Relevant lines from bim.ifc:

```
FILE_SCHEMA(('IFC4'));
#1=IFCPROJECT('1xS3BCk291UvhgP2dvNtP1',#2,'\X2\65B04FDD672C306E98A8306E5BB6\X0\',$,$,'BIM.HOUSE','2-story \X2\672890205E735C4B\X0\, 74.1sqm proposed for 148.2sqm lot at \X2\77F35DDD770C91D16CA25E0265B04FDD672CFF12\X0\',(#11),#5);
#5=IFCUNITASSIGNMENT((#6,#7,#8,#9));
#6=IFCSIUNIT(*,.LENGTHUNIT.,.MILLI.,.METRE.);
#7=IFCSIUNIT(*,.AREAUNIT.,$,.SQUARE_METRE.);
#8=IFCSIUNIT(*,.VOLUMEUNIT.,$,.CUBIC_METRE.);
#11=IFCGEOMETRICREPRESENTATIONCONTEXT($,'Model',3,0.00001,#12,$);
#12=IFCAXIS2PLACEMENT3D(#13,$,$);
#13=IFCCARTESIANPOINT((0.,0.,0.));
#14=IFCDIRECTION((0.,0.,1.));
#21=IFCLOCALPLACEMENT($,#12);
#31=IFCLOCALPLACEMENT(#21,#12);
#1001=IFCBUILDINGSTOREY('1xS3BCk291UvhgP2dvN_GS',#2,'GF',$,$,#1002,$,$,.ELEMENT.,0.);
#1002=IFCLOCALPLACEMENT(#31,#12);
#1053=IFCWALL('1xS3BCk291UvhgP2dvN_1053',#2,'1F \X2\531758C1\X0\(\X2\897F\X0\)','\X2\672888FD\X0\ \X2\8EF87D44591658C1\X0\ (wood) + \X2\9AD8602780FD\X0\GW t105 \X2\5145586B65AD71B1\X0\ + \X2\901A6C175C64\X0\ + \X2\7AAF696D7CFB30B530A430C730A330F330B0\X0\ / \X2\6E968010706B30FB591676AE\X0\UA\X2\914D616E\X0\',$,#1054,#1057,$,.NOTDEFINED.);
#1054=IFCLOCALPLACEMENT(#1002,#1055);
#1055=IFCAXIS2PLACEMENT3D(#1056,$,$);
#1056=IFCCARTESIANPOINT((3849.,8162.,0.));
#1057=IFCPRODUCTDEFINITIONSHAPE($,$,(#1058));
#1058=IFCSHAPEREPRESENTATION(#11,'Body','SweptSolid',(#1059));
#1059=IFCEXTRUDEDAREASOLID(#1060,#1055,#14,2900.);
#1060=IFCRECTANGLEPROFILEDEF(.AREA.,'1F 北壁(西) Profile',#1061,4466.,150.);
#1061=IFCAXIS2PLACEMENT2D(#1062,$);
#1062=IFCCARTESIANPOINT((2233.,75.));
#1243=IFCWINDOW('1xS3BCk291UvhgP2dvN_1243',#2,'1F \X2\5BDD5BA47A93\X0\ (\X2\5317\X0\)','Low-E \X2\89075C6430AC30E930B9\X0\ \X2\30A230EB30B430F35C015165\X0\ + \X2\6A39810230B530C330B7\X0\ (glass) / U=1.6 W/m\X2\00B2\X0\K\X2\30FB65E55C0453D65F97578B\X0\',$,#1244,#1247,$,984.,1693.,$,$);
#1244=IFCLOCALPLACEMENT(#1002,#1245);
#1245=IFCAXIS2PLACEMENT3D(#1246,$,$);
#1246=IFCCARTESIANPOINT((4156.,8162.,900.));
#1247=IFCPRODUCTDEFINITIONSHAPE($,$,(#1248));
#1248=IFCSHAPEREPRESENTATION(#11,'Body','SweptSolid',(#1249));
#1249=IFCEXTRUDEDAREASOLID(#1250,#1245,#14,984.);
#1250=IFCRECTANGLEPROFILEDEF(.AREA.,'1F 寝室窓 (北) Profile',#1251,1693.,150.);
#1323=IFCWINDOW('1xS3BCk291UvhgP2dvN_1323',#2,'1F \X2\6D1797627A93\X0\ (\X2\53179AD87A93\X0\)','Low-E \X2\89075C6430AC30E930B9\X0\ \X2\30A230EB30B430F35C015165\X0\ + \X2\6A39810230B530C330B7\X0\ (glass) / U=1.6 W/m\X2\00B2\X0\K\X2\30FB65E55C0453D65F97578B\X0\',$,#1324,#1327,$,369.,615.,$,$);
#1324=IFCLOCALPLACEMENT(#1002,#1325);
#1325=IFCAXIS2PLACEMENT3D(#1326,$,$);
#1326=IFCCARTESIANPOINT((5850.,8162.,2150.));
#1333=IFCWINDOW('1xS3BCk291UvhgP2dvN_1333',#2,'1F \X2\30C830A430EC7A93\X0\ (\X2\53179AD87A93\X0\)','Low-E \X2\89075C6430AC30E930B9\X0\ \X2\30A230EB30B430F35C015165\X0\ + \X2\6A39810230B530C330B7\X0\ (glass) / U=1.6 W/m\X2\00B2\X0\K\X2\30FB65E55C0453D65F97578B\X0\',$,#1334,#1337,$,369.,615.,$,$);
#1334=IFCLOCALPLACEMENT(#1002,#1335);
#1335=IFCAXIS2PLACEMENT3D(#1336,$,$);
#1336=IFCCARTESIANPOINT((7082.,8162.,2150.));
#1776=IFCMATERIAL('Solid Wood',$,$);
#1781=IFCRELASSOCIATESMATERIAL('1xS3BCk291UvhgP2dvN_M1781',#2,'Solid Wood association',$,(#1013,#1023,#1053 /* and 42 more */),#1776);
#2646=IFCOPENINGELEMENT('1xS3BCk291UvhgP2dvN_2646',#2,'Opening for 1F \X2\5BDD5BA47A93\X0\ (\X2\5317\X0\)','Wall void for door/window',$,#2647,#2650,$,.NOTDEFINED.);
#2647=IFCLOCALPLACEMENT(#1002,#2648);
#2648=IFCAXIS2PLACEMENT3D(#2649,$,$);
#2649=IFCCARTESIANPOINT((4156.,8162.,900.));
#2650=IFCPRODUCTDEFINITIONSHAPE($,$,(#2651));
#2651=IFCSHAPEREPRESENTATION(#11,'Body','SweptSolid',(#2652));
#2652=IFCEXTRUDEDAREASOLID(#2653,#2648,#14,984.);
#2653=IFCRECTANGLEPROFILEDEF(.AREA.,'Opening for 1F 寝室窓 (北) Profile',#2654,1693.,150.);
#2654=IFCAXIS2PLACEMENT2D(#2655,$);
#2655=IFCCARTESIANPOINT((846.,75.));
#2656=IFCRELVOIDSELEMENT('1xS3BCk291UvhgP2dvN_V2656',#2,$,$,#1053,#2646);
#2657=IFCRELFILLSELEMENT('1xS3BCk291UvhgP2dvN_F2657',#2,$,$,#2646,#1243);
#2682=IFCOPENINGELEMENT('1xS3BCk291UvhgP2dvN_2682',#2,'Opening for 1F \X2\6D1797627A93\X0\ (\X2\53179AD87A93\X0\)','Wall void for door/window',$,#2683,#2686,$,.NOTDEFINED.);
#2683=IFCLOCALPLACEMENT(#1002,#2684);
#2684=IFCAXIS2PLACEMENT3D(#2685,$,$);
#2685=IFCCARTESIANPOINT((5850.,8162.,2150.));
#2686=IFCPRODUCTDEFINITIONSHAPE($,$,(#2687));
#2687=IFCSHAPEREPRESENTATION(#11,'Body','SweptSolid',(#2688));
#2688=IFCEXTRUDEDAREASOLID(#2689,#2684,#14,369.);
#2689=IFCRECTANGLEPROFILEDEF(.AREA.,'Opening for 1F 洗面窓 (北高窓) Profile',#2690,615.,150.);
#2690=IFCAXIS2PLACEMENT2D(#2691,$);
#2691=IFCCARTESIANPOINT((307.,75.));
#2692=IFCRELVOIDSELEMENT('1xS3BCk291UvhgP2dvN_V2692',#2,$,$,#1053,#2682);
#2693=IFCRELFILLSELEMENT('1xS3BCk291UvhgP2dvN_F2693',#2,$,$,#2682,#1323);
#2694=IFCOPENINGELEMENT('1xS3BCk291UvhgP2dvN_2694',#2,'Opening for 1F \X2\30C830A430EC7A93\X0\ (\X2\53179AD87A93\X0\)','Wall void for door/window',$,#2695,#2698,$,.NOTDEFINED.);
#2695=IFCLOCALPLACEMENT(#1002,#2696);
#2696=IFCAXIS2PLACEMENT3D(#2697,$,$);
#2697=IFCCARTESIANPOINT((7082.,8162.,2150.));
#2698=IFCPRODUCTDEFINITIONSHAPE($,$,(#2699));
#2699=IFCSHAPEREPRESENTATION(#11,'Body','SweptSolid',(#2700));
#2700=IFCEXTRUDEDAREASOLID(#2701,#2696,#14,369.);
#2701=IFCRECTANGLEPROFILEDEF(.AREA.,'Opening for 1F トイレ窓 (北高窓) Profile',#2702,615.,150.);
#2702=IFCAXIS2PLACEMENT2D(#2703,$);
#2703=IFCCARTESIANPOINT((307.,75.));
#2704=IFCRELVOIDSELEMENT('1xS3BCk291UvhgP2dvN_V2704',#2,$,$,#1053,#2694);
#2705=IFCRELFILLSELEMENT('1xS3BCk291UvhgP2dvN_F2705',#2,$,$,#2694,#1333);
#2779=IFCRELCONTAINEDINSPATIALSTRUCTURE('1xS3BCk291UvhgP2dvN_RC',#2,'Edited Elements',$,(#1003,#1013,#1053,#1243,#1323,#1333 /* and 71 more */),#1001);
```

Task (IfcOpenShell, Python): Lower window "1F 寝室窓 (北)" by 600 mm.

```python
import numpy as np
import ifcopenshell
import ifcopenshell.api.geometry
import ifcopenshell.util.placement
import ifcopenshell.util.unit

model = ifcopenshell.open("bim.ifc")
unit_scale = ifcopenshell.util.unit.calculate_unit_scale(model)

window = model.by_id(1243)
opening = window.FillsVoids[0].RelatingOpeningElement
dz = -0.6 / unit_scale

shift = np.array([0.0, 0.0, dz])
# The window is not placed relative to its opening, so move both.
for product in (opening, window):
    matrix = ifcopenshell.util.placement.get_local_placement(product.ObjectPlacement)
    matrix[:3, 3] += shift
    ifcopenshell.api.geometry.edit_object_placement(model, product=product, matrix=matrix, is_si=False)

print(f"moved by {dz * unit_scale:+.3f} m")

model.write("bim_v2.ifc")
```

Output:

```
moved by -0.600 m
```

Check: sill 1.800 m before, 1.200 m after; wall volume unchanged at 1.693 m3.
